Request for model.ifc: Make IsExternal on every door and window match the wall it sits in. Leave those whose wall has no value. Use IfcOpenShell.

First a look at what the model holds.

```python
import ifcopenshell
import ifcopenshell.util.element

model = ifcopenshell.open("model.ifc")
print(model.schema)
seen = {}
for e in model.by_type("IfcDoor") + model.by_type("IfcWindow"):
    if not e.FillsVoids:
        continue
    host = e.FillsVoids[0].RelatingOpeningElement.VoidsElements[0].RelatingBuildingElement
    own = ifcopenshell.util.element.get_pset(e, f"Pset_{e.is_a()[3:].removesuffix('StandardCase')}Common", "IsExternal")
    wall = ifcopenshell.util.element.get_pset(host, "Pset_WallCommon", "IsExternal")
    seen[e.is_a(), own, wall] = seen.get((e.is_a(), own, wall), 0) + 1
for (cls, own, wall), count in sorted(seen.items(), key=str):
    print(count, cls, "IsExternal:", own, "| host wall:", wall)
```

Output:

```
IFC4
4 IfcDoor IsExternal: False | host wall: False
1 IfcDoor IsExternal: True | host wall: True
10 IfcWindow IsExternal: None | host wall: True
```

```python
import ifcopenshell
import ifcopenshell.api.pset
import ifcopenshell.util.element

model = ifcopenshell.open("model.ifc")

count = 0
for ifc_class, pset_name in (("IfcDoor", "Pset_DoorCommon"), ("IfcWindow", "Pset_WindowCommon")):
    for e in model.by_type(ifc_class):
        if not e.FillsVoids:
            continue
        host = e.FillsVoids[0].RelatingOpeningElement.VoidsElements[0].RelatingBuildingElement
        external = ifcopenshell.util.element.get_pset(host, "Pset_WallCommon", "IsExternal")
        if external is None or ifcopenshell.util.element.get_pset(e, pset_name, "IsExternal") == external:
            continue
        pset = ifcopenshell.api.pset.add_pset(model, product=e, name=pset_name)
        ifcopenshell.api.pset.edit_pset(model, pset=pset, properties={"IsExternal": external})
        count += 1

print(count, "updated")

model.write("model_edited.ifc")
```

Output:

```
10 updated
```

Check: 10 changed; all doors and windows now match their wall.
